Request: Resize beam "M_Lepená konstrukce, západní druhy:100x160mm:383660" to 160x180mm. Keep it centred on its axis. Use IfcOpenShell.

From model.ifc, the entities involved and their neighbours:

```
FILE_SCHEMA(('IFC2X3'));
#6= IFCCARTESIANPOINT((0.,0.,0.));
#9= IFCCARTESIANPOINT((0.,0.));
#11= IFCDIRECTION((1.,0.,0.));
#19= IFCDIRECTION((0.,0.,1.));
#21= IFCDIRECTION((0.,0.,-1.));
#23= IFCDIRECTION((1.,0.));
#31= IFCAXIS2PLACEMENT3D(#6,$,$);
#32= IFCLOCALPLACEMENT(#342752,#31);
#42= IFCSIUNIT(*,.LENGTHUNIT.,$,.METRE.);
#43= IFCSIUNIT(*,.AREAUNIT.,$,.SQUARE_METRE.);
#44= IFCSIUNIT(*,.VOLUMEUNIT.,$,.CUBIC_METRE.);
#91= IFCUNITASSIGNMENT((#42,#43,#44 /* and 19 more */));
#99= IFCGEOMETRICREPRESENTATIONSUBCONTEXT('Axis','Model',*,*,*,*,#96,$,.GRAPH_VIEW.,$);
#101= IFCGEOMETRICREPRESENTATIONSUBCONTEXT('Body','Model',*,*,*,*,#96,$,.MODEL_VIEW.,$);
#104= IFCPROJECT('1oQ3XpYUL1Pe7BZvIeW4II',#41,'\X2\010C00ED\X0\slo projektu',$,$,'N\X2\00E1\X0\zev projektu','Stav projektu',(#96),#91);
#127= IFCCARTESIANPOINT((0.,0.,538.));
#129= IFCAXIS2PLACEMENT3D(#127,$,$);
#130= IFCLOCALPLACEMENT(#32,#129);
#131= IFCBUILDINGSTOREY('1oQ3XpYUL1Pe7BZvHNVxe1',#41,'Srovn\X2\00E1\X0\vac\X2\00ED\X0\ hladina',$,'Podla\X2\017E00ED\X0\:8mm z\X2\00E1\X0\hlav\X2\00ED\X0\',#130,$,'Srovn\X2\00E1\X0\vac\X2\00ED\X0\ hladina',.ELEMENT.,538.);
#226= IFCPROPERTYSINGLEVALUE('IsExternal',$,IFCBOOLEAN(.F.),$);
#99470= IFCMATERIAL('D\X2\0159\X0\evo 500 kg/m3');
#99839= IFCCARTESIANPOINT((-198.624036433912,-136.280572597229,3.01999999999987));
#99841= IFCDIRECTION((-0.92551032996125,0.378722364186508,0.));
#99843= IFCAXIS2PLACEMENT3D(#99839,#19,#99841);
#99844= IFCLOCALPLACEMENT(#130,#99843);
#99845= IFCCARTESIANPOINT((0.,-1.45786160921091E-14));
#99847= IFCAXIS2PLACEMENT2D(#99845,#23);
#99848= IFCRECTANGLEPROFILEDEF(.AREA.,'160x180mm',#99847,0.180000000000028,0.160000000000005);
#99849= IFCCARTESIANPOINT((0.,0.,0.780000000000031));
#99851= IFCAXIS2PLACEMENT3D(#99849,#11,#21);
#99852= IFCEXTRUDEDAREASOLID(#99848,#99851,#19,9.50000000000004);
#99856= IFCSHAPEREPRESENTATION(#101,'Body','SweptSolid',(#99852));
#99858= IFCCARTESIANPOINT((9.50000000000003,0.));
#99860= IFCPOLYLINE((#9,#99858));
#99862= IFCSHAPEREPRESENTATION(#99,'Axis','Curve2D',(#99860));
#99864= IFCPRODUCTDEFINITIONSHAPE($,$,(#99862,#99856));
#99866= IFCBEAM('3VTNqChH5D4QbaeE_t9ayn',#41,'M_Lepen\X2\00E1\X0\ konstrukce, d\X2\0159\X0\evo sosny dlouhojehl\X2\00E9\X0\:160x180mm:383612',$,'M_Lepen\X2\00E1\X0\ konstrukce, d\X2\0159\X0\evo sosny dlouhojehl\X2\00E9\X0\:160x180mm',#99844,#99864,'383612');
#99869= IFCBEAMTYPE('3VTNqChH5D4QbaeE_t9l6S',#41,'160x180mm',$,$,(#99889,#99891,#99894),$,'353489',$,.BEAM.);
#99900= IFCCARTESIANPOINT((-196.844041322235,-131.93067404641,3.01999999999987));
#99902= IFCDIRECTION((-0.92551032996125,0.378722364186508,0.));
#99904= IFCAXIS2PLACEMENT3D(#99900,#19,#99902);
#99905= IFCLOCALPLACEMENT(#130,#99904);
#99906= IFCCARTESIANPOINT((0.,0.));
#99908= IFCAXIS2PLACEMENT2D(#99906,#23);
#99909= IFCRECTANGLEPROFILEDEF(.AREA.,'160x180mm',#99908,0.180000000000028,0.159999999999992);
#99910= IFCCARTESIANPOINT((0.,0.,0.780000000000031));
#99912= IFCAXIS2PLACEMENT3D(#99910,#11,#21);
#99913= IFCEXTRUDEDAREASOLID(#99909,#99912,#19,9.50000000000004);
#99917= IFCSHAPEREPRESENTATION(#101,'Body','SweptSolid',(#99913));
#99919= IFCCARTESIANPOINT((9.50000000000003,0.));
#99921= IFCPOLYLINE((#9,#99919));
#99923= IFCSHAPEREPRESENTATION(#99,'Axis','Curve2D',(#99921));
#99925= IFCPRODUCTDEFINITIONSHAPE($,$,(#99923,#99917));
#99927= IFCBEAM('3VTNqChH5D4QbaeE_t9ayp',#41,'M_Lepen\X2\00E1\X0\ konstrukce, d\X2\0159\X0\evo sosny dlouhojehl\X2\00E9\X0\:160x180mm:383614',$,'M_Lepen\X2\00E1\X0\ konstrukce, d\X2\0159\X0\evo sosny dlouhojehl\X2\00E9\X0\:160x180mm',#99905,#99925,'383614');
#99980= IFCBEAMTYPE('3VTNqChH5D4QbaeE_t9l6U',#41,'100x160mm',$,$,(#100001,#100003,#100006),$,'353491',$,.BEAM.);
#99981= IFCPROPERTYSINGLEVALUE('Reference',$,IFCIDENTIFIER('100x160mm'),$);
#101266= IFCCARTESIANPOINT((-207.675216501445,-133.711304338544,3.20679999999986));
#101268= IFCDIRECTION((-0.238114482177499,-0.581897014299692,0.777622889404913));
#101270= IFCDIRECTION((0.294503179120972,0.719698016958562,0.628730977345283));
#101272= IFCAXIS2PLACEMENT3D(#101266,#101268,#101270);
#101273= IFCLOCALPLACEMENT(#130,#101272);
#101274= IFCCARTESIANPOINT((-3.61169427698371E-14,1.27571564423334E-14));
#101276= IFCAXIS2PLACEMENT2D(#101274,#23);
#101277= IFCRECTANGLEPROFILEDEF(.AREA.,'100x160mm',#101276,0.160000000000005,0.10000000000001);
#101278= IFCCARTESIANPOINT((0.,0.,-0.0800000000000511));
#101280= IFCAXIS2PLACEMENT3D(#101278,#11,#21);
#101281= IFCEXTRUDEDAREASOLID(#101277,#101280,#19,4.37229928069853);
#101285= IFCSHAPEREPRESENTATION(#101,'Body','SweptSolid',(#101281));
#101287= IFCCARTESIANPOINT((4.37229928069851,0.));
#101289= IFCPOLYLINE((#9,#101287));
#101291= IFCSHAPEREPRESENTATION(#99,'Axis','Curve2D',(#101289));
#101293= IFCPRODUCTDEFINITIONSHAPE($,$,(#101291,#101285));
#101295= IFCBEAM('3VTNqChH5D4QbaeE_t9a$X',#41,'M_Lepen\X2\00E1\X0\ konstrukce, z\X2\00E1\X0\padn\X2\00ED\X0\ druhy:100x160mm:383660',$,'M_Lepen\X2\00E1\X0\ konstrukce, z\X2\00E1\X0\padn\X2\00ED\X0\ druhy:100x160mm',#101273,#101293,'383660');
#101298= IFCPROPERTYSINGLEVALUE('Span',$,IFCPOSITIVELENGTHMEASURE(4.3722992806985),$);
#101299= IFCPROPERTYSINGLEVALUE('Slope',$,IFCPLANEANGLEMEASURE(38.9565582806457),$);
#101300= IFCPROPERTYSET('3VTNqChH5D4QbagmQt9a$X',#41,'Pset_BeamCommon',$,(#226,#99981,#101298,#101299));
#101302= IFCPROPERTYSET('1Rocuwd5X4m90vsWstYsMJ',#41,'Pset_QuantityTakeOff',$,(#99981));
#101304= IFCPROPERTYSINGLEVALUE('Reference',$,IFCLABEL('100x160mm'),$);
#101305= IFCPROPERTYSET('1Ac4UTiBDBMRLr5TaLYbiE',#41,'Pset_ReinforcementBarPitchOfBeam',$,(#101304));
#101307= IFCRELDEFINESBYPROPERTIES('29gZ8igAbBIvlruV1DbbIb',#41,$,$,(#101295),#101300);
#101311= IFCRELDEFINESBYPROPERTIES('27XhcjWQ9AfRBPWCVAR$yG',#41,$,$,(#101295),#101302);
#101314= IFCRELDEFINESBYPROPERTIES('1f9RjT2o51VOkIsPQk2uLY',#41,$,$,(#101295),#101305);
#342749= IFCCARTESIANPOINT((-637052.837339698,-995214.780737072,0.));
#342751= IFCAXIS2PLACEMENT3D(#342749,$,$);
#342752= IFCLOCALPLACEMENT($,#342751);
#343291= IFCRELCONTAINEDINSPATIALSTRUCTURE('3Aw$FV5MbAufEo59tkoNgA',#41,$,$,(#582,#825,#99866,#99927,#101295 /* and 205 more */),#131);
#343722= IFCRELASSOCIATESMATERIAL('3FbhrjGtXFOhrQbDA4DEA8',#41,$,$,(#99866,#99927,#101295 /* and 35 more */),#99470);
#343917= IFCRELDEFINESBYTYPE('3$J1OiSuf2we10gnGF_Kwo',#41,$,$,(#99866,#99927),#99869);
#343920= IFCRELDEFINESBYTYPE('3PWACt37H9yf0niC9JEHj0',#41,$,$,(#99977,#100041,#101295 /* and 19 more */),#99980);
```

```python
import ifcopenshell
import ifcopenshell.api.pset
import ifcopenshell.api.type
import ifcopenshell.util.element
import ifcopenshell.util.representation

model = ifcopenshell.open("model.ifc")

member = model.by_guid("3VTNqChH5D4QbaeE_t9a$X")
source = next(p for p in model.by_type("IfcRectangleProfileDef") if p.ProfileName == "160x180mm")

body = ifcopenshell.util.representation.get_representation(member, "Model", "Body")
solid = body.Items[0]
old_profile = solid.SweptArea

# Copy the section's sizes but keep this member's own profile position.
profile = ifcopenshell.util.element.copy(model, source)
profile.Position = old_profile.Position
solid.SweptArea = profile
if not model.get_total_inverses(old_profile):
    ifcopenshell.util.element.remove_deep2(model, old_profile)

new_type = model.by_id(99869)
ifcopenshell.api.type.assign_type(
    model, related_objects=[member], relating_type=new_type, should_map_representations=False
)
member.Name = member.Name.replace("100x160mm", "160x180mm")
member.ObjectType = "M_Lepená konstrukce, západní druhy:160x180mm"
pset = model.by_id(ifcopenshell.util.element.get_pset(member, "Pset_BeamCommon", should_inherit=False)["id"])
ifcopenshell.api.pset.edit_pset(model, pset=pset, properties={"Reference": "160x180mm"})
pset = model.by_id(ifcopenshell.util.element.get_pset(member, "Pset_QuantityTakeOff", should_inherit=False)["id"])
ifcopenshell.api.pset.edit_pset(model, pset=pset, properties={"Reference": "160x180mm"})
pset = model.by_id(ifcopenshell.util.element.get_pset(member, "Pset_ReinforcementBarPitchOfBeam", should_inherit=False)["id"])
ifcopenshell.api.pset.edit_pset(model, pset=pset, properties={"Reference": "160x180mm"})

print(solid.SweptArea)

model.write("model_edited.ifc")
```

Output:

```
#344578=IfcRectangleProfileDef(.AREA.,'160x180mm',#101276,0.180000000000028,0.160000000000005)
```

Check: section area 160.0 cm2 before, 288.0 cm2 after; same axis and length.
